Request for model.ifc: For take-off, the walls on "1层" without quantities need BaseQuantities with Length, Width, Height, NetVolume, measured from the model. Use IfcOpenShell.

First a look at what the model holds.

```python
import ifcopenshell
import ifcopenshell.util.element
import ifcopenshell.util.unit

model = ifcopenshell.open("model.ifc")
print(model.schema)
for unit_type in ("LENGTHUNIT", "AREAUNIT", "VOLUMEUNIT"):
    print(unit_type, ifcopenshell.util.unit.calculate_unit_scale(model, unit_type))
storey = next(s for s in model.by_type("IfcBuildingStorey") if s.Name == "1层")
walls = [e for e in ifcopenshell.util.element.get_decomposition(storey) if e.is_a("IfcWall")]
for e in sorted(walls, key=lambda e: e.id()):
    print(e.id(), e.is_a(), e.Name, list(ifcopenshell.util.element.get_psets(e, qtos_only=True)), sep=" | ")
```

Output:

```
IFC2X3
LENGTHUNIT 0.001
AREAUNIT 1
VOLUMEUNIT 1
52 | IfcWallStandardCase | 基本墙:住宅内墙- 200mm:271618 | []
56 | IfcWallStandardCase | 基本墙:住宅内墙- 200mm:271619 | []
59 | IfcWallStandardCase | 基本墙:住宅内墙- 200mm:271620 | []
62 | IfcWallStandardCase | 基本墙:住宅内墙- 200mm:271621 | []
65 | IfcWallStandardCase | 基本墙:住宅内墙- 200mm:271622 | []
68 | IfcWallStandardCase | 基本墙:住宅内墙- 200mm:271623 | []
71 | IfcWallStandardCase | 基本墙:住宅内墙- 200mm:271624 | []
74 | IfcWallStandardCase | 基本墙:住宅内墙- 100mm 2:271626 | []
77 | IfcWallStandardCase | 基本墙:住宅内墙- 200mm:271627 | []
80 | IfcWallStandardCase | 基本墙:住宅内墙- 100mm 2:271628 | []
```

```python
import ifcopenshell
import ifcopenshell.api.pset
import ifcopenshell.geom
import ifcopenshell.util.element
import ifcopenshell.util.shape
import ifcopenshell.util.unit

model = ifcopenshell.open("model.ifc")
unit_scale = ifcopenshell.util.unit.calculate_unit_scale(model)
volume_scale = ifcopenshell.util.unit.calculate_unit_scale(model, "VOLUMEUNIT")
settings = ifcopenshell.geom.settings()

storey = next(s for s in model.by_type("IfcBuildingStorey") if s.Name == "1层")
walls = [e for e in ifcopenshell.util.element.get_decomposition(storey) if e.is_a("IfcWall")]

for e in sorted(walls, key=lambda e: e.id()):
    if ifcopenshell.util.element.get_psets(e, qtos_only=True, should_inherit=False):
        continue
    # Geometry comes back in metres, in the element's own axes.
    shape = ifcopenshell.geom.create_shape(settings, e)
    values = {
        "Length": ifcopenshell.util.shape.get_x(shape.geometry) / unit_scale,
        "Width": ifcopenshell.util.shape.get_y(shape.geometry) / unit_scale,
        "Height": ifcopenshell.util.shape.get_z(shape.geometry) / unit_scale,
        "NetVolume": ifcopenshell.util.shape.get_volume(shape.geometry) / volume_scale,
    }
    qto = ifcopenshell.api.pset.add_qto(model, product=e, name="BaseQuantities")
    ifcopenshell.api.pset.edit_qto(model, qto=qto, properties=values)
    print(e.id(), {k: round(v, 3) for k, v in values.items()})

model.write("model_v2.ifc")
```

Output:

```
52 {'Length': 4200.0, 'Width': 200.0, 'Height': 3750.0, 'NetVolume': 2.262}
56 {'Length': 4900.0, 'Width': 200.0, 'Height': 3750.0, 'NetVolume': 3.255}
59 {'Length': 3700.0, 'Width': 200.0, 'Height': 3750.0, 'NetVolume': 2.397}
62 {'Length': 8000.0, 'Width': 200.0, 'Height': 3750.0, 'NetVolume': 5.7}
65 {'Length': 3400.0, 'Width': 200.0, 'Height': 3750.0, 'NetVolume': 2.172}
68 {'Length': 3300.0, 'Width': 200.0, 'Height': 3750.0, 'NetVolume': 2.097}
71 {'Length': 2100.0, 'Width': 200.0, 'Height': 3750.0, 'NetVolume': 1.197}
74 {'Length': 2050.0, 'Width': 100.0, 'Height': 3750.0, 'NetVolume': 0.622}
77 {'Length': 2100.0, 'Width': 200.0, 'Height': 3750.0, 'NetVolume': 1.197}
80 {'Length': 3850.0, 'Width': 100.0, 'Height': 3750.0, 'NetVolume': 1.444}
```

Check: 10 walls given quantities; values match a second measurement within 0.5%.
